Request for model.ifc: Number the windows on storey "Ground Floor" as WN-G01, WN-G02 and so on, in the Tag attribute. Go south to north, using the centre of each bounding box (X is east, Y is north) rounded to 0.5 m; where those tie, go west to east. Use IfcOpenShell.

First a look at what the model holds.

```python
import ifcopenshell
import ifcopenshell.util.element
import ifcopenshell.util.placement

model = ifcopenshell.open("model.ifc")
print(model.schema)
storey = next(s for s in model.by_type("IfcBuildingStorey") if s.Name == "Ground Floor")
windows = [e for e in ifcopenshell.util.element.get_decomposition(storey) if e.is_a("IfcWindow")]
for e in sorted(windows, key=lambda e: e.id()):
    origin = ifcopenshell.util.placement.get_local_placement(e.ObjectPlacement)[:3, 3]
    print(e.id(), e.Tag, e.Name, origin.round(2) + 0.0, sep=" | ")
```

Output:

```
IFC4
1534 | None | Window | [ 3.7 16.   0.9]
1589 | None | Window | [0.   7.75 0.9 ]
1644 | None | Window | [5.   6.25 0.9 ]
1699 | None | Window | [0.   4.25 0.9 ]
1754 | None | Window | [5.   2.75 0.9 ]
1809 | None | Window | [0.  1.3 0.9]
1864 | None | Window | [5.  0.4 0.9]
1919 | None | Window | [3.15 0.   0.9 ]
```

```python
import ifcopenshell
import ifcopenshell.geom
import ifcopenshell.util.element
import ifcopenshell.util.shape

model = ifcopenshell.open("model.ifc")
settings = ifcopenshell.geom.settings()
settings.set("use-world-coords", True)


def centre(element):
    shape = ifcopenshell.geom.create_shape(settings, element)
    return ifcopenshell.util.shape.get_bbox_centroid(shape.geometry)


storey = next(s for s in model.by_type("IfcBuildingStorey") if s.Name == "Ground Floor")
windows = [e for e in ifcopenshell.util.element.get_decomposition(storey) if e.is_a("IfcWindow")]

# Insertion points can sit at a corner or the storey origin, so sort by the geometry (in metres).
centres = {e: centre(e) for e in windows}
windows.sort(key=lambda e: (round(centres[e][1] / 0.5), centres[e][0]))

for i, e in enumerate(windows, start=1):
    number = f"WN-G{i:02d}"
    e.Tag = number
    print(e.id(), number)

model.write("model_updated.ifc")
```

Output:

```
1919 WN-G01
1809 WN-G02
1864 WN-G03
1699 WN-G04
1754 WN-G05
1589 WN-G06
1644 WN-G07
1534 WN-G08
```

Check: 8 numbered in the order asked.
